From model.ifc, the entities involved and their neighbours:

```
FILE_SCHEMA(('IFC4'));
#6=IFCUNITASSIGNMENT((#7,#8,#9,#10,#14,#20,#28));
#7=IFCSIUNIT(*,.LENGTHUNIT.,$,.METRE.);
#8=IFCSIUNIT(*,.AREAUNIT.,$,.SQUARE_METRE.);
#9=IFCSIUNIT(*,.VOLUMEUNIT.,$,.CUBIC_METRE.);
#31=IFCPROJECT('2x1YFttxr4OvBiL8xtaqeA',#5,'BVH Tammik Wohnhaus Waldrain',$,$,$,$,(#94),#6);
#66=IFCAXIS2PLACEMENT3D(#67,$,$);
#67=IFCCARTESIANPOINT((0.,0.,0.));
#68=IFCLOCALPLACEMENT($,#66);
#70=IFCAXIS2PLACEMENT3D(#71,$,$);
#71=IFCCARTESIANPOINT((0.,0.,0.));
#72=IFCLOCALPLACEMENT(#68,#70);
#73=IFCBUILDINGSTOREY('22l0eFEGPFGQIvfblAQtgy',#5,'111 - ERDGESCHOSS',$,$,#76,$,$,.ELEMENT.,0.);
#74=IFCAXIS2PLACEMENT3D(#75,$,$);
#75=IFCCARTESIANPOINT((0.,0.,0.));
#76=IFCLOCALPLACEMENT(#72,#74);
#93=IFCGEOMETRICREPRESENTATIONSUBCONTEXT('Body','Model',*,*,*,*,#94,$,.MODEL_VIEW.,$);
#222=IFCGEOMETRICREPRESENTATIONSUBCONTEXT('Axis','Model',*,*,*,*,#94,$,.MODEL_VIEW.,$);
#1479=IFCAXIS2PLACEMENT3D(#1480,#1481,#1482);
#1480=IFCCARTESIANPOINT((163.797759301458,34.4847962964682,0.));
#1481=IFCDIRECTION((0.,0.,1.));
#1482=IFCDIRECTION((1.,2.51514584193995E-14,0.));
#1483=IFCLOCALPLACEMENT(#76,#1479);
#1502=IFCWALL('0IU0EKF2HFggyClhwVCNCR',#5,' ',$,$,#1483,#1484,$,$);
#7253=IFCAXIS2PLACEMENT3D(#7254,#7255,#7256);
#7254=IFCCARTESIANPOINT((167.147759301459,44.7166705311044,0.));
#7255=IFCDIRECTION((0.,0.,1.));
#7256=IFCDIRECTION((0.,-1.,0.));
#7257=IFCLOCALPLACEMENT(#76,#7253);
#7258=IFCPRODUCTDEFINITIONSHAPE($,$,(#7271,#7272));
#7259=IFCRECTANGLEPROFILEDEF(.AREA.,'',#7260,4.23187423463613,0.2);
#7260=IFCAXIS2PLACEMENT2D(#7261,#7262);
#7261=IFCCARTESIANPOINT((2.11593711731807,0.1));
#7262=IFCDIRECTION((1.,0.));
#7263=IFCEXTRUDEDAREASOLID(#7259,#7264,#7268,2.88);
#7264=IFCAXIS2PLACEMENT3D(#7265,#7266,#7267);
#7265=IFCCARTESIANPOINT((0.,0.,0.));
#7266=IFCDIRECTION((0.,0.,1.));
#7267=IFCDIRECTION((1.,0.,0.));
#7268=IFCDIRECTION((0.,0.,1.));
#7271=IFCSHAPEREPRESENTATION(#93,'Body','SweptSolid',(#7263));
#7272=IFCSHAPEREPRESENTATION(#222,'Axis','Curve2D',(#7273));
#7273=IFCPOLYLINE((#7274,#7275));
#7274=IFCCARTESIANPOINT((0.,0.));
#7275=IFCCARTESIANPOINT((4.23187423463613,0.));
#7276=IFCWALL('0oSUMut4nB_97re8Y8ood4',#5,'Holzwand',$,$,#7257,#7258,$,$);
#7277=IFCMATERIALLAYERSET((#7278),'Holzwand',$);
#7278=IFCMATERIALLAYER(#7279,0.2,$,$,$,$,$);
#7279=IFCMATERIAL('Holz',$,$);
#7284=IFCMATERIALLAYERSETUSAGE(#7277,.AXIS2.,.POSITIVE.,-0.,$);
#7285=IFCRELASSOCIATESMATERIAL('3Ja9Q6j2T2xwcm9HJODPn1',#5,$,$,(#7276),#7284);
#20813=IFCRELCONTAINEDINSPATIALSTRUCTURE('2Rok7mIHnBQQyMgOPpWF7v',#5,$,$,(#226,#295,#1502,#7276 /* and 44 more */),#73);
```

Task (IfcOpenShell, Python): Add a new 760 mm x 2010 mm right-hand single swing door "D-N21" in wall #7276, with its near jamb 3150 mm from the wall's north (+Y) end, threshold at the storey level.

```python
import numpy as np
import ifcopenshell
import ifcopenshell.api.feature
import ifcopenshell.api.geometry
import ifcopenshell.api.root
import ifcopenshell.api.spatial
import ifcopenshell.geom
import ifcopenshell.util.element
import ifcopenshell.util.placement
import ifcopenshell.util.representation
import ifcopenshell.util.shape
import ifcopenshell.util.unit

model = ifcopenshell.open("model.ifc")
unit_scale = ifcopenshell.util.unit.calculate_unit_scale(model)
settings = ifcopenshell.geom.settings()


def volume(element):
    """Net volume in cubic metres, openings subtracted."""
    shape = ifcopenshell.geom.create_shape(settings, element)
    return ifcopenshell.util.shape.get_volume(shape.geometry)


wall = model.by_guid("0oSUMut4nB_97re8Y8ood4")
storey = ifcopenshell.util.element.get_container(wall, ifc_class="IfcBuildingStorey")
context = ifcopenshell.util.representation.get_context(model, "Model", "Body", "MODEL_VIEW")
before = volume(wall)

width, height, from_end, sill = 0.76, 2.01, 3.15, 0.0  # metres

# The wall runs along its own X axis, and the end named is its -X end.
wall_shape = ifcopenshell.geom.create_shape(settings, wall)
x, y, z = ifcopenshell.util.shape.get_vertices(wall_shape.geometry).T
start = x.min() + from_end
face, thickness = float(y.min()), float(y.max() - y.min())
wall_matrix = ifcopenshell.util.placement.get_local_placement(wall.ObjectPlacement)
level = ifcopenshell.util.placement.get_local_placement(storey.ObjectPlacement)[2, 3]


def in_wall(x, y):
    """Placement at x, y metres in the wall's axes, at sill height."""
    matrix = wall_matrix.copy()
    matrix[:, 3] = wall_matrix @ np.array([x / unit_scale, y / unit_scale, 0.0, 1.0])
    matrix[2, 3] = level + sill / unit_scale
    return matrix


# Opening: a box that overshoots both wall faces by 50 mm.
opening = ifcopenshell.api.root.create_entity(model, ifc_class="IfcOpeningElement", predefined_type="OPENING")
box = ifcopenshell.api.geometry.add_wall_representation(
    model, context=context, length=width, height=height, thickness=thickness + 0.1
)
ifcopenshell.api.geometry.assign_representation(model, product=opening, representation=box)
ifcopenshell.api.geometry.edit_object_placement(model, product=opening, matrix=in_wall(start, face - 0.05), is_si=False)
ifcopenshell.api.feature.add_feature(model, feature=opening, element=wall)

door = ifcopenshell.api.root.create_entity(model, ifc_class="IfcDoor", name="D-N21", predefined_type="DOOR")
door.OverallWidth, door.OverallHeight = width / unit_scale, height / unit_scale
door.OperationType = "SINGLE_SWING_RIGHT"
body = ifcopenshell.api.geometry.add_door_representation(
    model,
    context=context,
    overall_width=door.OverallWidth,
    overall_height=door.OverallHeight,
    operation_type="SINGLE_SWING_RIGHT",
    lining_properties={"LiningDepth": thickness / unit_scale, "ThresholdDepth": thickness / unit_scale},
)
ifcopenshell.api.geometry.assign_representation(model, product=door, representation=body)
ifcopenshell.api.spatial.assign_container(model, products=[door], relating_structure=storey)
ifcopenshell.api.feature.add_filling(model, opening=opening, element=door)

# The lining spans the wall, so the door starts at the wall face.
ifcopenshell.api.geometry.edit_object_placement(model, product=door, matrix=in_wall(start, face), is_si=False)

after = volume(wall)

print(f"wall volume {before:.3f} -> {after:.3f} m3")

model.write("model_edited.ifc")
```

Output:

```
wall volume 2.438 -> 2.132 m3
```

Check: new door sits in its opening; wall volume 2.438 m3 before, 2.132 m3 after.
